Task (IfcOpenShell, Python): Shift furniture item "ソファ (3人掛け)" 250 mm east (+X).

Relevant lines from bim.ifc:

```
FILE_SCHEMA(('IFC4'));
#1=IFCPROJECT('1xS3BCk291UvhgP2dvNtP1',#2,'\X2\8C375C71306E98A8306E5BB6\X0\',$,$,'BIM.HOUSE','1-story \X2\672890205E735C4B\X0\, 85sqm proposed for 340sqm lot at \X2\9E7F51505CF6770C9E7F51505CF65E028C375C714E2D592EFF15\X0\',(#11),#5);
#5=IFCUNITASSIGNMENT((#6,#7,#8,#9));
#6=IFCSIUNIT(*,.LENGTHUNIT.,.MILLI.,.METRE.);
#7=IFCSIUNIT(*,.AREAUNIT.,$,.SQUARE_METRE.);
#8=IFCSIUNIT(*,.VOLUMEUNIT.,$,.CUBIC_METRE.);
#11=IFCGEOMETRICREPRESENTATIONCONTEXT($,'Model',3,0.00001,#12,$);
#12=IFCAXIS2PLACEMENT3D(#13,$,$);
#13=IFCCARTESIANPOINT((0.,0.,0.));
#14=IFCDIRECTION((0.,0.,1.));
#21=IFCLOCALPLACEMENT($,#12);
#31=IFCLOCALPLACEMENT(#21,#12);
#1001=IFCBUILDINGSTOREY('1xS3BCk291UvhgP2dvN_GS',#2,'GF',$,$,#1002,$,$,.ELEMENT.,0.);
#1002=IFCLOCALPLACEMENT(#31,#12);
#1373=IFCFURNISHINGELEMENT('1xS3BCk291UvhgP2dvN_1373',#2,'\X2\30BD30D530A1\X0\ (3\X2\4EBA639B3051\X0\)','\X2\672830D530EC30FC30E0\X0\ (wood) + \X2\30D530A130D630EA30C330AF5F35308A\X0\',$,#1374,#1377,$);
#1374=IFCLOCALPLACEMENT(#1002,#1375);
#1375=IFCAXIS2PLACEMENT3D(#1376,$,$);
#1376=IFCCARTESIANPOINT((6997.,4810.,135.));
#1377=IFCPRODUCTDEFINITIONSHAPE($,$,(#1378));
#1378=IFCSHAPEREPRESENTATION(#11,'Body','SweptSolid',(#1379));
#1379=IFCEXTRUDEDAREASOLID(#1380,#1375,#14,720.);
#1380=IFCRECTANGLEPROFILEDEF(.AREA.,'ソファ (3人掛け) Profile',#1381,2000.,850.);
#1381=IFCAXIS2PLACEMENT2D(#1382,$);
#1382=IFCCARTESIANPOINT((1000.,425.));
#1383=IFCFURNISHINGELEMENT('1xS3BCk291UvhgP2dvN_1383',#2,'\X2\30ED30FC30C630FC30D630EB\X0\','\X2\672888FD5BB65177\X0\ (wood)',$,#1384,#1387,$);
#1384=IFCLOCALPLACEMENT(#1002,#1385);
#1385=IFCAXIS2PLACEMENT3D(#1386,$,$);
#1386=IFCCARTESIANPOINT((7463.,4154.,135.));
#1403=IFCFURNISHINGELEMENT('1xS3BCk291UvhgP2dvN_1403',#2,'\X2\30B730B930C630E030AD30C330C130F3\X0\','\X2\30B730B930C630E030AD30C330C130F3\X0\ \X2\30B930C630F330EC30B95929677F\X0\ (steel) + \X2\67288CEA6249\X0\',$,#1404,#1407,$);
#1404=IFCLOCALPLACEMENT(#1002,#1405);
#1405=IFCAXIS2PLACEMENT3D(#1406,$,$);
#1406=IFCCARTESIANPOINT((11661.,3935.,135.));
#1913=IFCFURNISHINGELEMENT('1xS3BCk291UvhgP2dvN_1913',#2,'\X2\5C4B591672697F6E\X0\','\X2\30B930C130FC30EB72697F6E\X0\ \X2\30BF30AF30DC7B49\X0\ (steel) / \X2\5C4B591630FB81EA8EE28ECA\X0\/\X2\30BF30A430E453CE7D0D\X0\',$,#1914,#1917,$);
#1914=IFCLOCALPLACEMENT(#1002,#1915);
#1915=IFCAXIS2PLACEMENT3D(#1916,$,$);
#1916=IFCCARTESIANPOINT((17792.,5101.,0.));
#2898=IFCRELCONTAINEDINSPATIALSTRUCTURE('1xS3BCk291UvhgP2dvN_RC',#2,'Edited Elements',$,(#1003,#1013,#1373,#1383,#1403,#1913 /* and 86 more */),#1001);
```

```python
import ifcopenshell
import ifcopenshell.api.geometry
import ifcopenshell.util.placement

model = ifcopenshell.open("bim.ifc")

item = model.by_guid("1xS3BCk291UvhgP2dvN_1373")
matrix = ifcopenshell.util.placement.get_local_placement(item.ObjectPlacement)
matrix[0, 3] += 250.0
ifcopenshell.api.geometry.edit_object_placement(model, product=item, matrix=matrix, is_si=False)

print(ifcopenshell.util.placement.get_local_placement(item.ObjectPlacement).round(3) + 0.0)

model.write("bim_v2.ifc")
```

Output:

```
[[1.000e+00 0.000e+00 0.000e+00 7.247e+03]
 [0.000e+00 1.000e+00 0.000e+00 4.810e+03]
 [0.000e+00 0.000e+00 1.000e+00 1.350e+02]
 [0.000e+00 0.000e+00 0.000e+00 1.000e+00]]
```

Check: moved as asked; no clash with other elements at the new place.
